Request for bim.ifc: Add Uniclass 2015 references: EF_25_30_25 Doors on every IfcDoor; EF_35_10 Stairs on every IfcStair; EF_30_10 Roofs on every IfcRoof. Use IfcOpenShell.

First a look at what the model holds.

```python
import ifcopenshell

model = ifcopenshell.open("bim.ifc")
print(model.schema)
print("classifications:", [c.Name for c in model.by_type("IfcClassification")])
for ifc_class in ("IfcDoor", "IfcRoof", "IfcStair", "IfcWall", "IfcWindow"):
    print(ifc_class, len(model.by_type(ifc_class)))
```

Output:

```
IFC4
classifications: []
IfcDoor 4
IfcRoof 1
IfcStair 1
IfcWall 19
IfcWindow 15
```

```python
import ifcopenshell
import ifcopenshell.api.classification

model = ifcopenshell.open("bim.ifc")

system = ifcopenshell.api.classification.add_classification(model, classification="Uniclass 2015")

codes = {
    "IfcDoor": ("EF_25_30_25", "Doors"),
    "IfcStair": ("EF_35_10", "Stairs"),
    "IfcRoof": ("EF_30_10", "Roofs"),
}
for ifc_class, (code, name) in codes.items():
    products = model.by_type(ifc_class)
    ifcopenshell.api.classification.add_reference(
        model, products=products, classification=system, identification=code, name=name
    )
    print(code, len(products))

model.write("bim_edited.ifc")
```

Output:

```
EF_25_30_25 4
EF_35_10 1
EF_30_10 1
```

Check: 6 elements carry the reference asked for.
